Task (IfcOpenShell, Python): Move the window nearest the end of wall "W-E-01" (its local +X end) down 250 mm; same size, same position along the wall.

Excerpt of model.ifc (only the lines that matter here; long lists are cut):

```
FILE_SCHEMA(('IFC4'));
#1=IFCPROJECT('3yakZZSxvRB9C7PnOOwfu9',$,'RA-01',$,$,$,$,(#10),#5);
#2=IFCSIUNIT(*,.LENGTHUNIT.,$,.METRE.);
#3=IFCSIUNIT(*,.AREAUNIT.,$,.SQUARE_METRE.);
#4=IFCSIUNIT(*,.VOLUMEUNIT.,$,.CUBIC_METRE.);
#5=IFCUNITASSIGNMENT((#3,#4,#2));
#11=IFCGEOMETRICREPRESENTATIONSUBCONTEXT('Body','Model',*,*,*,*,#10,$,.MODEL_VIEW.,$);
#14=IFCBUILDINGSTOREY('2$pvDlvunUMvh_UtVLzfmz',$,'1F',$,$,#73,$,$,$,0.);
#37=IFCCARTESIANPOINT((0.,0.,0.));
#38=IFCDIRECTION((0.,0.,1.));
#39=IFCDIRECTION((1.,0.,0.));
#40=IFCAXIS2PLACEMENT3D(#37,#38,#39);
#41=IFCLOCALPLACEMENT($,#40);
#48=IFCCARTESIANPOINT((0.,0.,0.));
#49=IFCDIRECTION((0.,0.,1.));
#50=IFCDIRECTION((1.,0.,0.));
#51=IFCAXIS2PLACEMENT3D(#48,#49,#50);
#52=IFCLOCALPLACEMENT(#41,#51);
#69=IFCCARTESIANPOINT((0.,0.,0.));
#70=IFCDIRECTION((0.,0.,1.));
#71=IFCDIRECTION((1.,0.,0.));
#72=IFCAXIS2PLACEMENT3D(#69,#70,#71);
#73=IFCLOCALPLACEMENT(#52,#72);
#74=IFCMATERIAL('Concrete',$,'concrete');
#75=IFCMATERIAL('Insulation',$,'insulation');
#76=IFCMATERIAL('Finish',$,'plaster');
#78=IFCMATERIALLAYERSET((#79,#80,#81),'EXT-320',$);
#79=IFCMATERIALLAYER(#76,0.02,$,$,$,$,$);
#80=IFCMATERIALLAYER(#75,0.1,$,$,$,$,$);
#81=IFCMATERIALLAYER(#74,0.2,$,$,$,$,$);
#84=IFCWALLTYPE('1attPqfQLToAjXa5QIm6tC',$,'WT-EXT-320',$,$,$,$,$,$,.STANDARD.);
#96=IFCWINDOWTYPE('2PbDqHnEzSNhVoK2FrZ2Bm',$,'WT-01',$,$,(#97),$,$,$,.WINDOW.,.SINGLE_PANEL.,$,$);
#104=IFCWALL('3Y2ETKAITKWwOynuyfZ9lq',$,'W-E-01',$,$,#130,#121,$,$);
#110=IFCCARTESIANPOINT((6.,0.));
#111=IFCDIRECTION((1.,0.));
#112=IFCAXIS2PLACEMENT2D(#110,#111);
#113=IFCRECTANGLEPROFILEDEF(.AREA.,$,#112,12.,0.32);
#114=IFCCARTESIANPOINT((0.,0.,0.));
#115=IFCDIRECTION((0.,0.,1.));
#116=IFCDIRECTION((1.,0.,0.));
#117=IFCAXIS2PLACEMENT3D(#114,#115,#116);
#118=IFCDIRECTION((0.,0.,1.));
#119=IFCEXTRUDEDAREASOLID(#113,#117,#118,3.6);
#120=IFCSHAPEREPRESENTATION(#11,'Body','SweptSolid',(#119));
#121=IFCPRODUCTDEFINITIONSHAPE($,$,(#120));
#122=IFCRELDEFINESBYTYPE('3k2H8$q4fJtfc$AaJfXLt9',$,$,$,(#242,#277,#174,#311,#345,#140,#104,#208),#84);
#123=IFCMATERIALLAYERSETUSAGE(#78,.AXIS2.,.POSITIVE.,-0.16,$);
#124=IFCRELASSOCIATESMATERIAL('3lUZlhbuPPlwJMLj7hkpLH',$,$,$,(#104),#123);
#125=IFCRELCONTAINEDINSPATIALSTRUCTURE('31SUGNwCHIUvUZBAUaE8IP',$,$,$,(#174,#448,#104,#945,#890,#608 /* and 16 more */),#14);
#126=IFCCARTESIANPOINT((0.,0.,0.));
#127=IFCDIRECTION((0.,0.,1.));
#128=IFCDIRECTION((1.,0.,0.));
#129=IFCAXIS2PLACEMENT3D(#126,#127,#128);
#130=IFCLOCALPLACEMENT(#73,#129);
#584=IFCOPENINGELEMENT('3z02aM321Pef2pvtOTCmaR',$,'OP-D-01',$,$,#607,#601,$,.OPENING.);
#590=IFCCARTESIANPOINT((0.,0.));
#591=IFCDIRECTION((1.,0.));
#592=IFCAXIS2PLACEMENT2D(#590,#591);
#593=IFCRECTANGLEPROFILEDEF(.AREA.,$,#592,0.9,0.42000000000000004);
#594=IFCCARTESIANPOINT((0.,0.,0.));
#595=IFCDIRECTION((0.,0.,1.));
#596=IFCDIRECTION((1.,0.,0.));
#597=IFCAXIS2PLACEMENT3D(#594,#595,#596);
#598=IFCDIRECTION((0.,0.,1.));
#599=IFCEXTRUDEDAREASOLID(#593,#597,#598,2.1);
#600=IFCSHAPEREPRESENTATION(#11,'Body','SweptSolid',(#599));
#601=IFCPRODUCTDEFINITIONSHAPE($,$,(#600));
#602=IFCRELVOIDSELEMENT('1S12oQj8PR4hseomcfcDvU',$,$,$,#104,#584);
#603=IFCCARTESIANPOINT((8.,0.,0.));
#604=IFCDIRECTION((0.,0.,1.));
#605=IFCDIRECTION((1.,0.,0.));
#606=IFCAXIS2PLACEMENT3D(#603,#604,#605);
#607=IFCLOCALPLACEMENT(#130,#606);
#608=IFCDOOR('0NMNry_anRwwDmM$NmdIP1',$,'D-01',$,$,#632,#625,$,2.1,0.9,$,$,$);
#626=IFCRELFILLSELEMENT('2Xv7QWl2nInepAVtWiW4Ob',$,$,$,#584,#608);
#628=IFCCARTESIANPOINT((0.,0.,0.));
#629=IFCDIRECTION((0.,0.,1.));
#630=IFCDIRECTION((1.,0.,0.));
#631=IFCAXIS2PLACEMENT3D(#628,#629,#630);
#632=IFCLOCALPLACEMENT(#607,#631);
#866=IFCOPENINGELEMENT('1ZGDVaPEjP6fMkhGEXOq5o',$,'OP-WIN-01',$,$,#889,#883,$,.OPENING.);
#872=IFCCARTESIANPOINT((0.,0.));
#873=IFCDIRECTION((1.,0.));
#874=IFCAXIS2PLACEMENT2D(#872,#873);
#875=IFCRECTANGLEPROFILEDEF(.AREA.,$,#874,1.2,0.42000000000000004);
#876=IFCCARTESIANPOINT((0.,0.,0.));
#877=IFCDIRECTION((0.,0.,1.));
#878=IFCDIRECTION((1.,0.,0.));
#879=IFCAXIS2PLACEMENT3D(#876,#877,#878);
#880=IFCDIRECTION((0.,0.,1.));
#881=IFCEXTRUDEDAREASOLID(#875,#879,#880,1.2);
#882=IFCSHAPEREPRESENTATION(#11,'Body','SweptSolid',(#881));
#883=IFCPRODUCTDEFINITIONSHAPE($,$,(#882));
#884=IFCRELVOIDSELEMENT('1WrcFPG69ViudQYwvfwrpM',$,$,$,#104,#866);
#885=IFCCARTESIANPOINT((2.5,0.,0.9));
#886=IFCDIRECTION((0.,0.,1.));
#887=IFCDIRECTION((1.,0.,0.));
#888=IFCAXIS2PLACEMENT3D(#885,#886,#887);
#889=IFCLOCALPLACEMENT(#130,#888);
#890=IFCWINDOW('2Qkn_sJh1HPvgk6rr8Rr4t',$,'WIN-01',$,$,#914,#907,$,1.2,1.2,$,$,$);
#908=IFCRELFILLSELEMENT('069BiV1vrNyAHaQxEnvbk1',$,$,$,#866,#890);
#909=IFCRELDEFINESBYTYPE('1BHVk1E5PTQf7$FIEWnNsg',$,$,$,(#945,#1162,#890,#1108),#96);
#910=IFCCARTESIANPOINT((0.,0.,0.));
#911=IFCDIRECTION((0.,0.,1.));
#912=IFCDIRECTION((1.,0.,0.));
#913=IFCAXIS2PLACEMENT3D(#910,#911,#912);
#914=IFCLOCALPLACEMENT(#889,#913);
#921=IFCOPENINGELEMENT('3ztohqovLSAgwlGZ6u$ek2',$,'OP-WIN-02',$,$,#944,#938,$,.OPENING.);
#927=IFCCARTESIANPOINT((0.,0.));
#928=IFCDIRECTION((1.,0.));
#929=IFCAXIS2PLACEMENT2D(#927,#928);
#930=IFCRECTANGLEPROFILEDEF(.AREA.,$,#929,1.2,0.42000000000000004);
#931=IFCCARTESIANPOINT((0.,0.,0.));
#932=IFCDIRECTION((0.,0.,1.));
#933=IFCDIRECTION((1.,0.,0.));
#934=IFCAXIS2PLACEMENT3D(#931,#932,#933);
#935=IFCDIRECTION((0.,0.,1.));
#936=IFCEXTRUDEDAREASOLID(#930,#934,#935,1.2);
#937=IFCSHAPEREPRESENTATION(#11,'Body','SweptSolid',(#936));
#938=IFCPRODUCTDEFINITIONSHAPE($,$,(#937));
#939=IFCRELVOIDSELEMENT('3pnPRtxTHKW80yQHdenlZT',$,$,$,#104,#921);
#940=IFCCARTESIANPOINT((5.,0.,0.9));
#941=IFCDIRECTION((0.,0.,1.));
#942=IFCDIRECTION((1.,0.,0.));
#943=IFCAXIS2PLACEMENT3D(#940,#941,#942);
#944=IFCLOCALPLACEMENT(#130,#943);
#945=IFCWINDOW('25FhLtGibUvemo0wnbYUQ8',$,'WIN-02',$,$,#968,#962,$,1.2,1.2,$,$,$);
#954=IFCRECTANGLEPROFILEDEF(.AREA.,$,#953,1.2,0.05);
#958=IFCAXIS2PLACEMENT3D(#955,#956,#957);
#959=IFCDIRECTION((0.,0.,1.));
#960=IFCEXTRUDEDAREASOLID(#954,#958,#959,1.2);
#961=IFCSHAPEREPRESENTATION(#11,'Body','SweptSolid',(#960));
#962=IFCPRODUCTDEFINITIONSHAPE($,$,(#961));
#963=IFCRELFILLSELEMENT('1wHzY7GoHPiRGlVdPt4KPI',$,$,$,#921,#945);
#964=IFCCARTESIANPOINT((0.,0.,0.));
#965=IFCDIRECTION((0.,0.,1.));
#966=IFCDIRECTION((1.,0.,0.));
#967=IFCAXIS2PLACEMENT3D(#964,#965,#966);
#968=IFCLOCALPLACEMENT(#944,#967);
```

```python
import numpy as np
import ifcopenshell
import ifcopenshell.api.geometry
import ifcopenshell.util.placement
import ifcopenshell.util.unit

model = ifcopenshell.open("model.ifc")
unit_scale = ifcopenshell.util.unit.calculate_unit_scale(model)

window = model.by_id(945)
opening = window.FillsVoids[0].RelatingOpeningElement
dz = -0.25 / unit_scale

shift = np.array([0.0, 0.0, dz])
# The window is placed relative to its opening, so it follows when the opening moves.
matrix = ifcopenshell.util.placement.get_local_placement(opening.ObjectPlacement)
matrix[:3, 3] += shift
ifcopenshell.api.geometry.edit_object_placement(
    model, product=opening, matrix=matrix, is_si=False, should_transform_children=True
)

print(f"moved by {dz * unit_scale:+.3f} m")

model.write("model_edited.ifc")
```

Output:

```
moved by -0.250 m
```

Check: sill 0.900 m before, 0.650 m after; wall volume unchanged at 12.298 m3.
